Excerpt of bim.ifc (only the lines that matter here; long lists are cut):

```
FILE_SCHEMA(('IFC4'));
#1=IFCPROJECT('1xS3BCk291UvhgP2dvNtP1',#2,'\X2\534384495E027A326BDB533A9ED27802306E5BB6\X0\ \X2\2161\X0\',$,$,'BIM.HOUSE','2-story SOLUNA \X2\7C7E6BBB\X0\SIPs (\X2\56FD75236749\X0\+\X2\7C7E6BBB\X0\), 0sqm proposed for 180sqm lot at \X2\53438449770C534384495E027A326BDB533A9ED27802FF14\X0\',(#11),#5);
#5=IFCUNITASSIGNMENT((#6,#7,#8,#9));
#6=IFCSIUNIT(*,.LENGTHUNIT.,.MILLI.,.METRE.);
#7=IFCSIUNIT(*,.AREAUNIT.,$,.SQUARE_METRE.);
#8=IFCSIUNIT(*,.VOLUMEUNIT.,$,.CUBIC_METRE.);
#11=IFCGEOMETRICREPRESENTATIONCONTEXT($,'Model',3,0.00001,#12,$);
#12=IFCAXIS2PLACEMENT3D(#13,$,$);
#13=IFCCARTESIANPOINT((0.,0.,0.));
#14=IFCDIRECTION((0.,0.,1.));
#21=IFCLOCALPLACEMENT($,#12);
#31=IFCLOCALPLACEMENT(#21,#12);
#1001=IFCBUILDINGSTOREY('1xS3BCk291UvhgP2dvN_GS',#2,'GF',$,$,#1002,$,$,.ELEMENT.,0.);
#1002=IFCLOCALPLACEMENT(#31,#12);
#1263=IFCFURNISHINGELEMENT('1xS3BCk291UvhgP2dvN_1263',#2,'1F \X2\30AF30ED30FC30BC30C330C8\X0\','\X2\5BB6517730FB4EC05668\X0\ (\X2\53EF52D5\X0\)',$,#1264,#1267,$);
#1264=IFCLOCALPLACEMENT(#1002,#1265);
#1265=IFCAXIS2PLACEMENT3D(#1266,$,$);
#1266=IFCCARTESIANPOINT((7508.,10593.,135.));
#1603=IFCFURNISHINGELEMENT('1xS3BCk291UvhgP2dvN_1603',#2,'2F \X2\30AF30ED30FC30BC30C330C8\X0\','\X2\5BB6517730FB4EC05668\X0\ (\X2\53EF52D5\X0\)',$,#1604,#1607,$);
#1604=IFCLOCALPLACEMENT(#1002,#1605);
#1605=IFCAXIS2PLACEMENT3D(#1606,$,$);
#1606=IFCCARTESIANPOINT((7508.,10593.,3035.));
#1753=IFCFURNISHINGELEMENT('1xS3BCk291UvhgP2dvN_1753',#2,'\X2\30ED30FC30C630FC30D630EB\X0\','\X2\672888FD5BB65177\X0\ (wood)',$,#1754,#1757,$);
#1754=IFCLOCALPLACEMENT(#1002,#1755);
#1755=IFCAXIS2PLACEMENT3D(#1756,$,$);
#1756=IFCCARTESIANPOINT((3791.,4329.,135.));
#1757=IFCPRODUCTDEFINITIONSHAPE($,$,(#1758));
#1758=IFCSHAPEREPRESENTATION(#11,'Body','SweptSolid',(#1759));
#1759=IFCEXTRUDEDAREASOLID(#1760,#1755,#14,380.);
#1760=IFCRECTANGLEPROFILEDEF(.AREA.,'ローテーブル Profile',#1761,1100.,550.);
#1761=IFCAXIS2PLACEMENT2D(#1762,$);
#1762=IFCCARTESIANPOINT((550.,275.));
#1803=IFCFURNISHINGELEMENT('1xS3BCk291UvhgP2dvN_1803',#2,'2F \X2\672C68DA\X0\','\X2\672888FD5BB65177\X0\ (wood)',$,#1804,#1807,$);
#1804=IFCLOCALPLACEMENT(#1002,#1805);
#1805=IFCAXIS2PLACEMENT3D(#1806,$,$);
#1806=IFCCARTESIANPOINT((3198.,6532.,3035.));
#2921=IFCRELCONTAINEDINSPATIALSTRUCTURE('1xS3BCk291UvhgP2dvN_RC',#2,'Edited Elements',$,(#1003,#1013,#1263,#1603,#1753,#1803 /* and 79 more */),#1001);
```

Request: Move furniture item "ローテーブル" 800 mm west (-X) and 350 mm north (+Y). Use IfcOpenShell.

```python
import ifcopenshell
import ifcopenshell.api.geometry
import ifcopenshell.util.placement

model = ifcopenshell.open("bim.ifc")

item = model.by_guid("1xS3BCk291UvhgP2dvN_1753")
matrix = ifcopenshell.util.placement.get_local_placement(item.ObjectPlacement)
matrix[0, 3] -= 800.0
matrix[1, 3] += 350.0
ifcopenshell.api.geometry.edit_object_placement(model, product=item, matrix=matrix, is_si=False)

print(ifcopenshell.util.placement.get_local_placement(item.ObjectPlacement).round(3) + 0.0)

model.write("bim_v2.ifc")
```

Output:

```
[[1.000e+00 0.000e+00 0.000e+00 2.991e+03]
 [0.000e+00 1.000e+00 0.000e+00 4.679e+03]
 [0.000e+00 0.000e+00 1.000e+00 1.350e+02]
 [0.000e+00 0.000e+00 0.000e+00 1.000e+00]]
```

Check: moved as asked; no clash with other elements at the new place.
